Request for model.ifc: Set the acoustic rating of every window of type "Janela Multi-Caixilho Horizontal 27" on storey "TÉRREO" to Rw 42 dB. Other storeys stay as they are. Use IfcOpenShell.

First a look at what the model holds.

```python
import ifcopenshell
import ifcopenshell.util.element

model = ifcopenshell.open("model.ifc")
print(model.schema)
storey = next(s for s in model.by_type("IfcBuildingStorey") if s.Name == "TÉRREO")
windows = [e for e in ifcopenshell.util.element.get_decomposition(storey) if e.is_a("IfcWindow")]
seen = {}
for e in windows:
    element_type = ifcopenshell.util.element.get_type(e)
    key = (element_type.Name if element_type != e and element_type else None, ifcopenshell.util.element.get_pset(e, "Pset_WindowCommon", "AcousticRating"))
    seen[key] = seen.get(key, 0) + 1
for (name, value), count in sorted(seen.items(), key=str):
    print(count, "x", name, "|", value)
```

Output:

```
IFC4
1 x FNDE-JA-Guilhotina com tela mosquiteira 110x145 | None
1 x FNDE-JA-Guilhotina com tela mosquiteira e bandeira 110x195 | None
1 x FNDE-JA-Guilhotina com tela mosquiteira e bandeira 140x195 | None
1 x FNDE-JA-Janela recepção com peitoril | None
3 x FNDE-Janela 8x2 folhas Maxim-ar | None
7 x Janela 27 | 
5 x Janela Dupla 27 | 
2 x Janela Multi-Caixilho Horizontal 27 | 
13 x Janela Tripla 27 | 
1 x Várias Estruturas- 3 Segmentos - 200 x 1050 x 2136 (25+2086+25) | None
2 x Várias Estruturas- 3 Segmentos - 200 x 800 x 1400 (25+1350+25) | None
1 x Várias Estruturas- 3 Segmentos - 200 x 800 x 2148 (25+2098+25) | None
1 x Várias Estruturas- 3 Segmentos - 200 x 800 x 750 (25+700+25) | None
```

```python
import ifcopenshell
import ifcopenshell.api.pset
import ifcopenshell.util.element

model = ifcopenshell.open("model.ifc")

storey = next(s for s in model.by_type("IfcBuildingStorey") if s.Name == "TÉRREO")
windows = [e for e in ifcopenshell.util.element.get_decomposition(storey) if e.is_a("IfcWindow")]

count = 0
for e in windows:
    element_type = ifcopenshell.util.element.get_type(e)
    if element_type in (None, e) or element_type.Name != "Janela Multi-Caixilho Horizontal 27":
        continue
    # add_pset returns the element's existing set when there is one.
    pset = ifcopenshell.api.pset.add_pset(model, product=e, name="Pset_WindowCommon")
    ifcopenshell.api.pset.edit_pset(model, pset=pset, properties={"AcousticRating": "Rw 42 dB"})
    count += 1

print(count, "windows updated")

model.write("model_v2.ifc")
```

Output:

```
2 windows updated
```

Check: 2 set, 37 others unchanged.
